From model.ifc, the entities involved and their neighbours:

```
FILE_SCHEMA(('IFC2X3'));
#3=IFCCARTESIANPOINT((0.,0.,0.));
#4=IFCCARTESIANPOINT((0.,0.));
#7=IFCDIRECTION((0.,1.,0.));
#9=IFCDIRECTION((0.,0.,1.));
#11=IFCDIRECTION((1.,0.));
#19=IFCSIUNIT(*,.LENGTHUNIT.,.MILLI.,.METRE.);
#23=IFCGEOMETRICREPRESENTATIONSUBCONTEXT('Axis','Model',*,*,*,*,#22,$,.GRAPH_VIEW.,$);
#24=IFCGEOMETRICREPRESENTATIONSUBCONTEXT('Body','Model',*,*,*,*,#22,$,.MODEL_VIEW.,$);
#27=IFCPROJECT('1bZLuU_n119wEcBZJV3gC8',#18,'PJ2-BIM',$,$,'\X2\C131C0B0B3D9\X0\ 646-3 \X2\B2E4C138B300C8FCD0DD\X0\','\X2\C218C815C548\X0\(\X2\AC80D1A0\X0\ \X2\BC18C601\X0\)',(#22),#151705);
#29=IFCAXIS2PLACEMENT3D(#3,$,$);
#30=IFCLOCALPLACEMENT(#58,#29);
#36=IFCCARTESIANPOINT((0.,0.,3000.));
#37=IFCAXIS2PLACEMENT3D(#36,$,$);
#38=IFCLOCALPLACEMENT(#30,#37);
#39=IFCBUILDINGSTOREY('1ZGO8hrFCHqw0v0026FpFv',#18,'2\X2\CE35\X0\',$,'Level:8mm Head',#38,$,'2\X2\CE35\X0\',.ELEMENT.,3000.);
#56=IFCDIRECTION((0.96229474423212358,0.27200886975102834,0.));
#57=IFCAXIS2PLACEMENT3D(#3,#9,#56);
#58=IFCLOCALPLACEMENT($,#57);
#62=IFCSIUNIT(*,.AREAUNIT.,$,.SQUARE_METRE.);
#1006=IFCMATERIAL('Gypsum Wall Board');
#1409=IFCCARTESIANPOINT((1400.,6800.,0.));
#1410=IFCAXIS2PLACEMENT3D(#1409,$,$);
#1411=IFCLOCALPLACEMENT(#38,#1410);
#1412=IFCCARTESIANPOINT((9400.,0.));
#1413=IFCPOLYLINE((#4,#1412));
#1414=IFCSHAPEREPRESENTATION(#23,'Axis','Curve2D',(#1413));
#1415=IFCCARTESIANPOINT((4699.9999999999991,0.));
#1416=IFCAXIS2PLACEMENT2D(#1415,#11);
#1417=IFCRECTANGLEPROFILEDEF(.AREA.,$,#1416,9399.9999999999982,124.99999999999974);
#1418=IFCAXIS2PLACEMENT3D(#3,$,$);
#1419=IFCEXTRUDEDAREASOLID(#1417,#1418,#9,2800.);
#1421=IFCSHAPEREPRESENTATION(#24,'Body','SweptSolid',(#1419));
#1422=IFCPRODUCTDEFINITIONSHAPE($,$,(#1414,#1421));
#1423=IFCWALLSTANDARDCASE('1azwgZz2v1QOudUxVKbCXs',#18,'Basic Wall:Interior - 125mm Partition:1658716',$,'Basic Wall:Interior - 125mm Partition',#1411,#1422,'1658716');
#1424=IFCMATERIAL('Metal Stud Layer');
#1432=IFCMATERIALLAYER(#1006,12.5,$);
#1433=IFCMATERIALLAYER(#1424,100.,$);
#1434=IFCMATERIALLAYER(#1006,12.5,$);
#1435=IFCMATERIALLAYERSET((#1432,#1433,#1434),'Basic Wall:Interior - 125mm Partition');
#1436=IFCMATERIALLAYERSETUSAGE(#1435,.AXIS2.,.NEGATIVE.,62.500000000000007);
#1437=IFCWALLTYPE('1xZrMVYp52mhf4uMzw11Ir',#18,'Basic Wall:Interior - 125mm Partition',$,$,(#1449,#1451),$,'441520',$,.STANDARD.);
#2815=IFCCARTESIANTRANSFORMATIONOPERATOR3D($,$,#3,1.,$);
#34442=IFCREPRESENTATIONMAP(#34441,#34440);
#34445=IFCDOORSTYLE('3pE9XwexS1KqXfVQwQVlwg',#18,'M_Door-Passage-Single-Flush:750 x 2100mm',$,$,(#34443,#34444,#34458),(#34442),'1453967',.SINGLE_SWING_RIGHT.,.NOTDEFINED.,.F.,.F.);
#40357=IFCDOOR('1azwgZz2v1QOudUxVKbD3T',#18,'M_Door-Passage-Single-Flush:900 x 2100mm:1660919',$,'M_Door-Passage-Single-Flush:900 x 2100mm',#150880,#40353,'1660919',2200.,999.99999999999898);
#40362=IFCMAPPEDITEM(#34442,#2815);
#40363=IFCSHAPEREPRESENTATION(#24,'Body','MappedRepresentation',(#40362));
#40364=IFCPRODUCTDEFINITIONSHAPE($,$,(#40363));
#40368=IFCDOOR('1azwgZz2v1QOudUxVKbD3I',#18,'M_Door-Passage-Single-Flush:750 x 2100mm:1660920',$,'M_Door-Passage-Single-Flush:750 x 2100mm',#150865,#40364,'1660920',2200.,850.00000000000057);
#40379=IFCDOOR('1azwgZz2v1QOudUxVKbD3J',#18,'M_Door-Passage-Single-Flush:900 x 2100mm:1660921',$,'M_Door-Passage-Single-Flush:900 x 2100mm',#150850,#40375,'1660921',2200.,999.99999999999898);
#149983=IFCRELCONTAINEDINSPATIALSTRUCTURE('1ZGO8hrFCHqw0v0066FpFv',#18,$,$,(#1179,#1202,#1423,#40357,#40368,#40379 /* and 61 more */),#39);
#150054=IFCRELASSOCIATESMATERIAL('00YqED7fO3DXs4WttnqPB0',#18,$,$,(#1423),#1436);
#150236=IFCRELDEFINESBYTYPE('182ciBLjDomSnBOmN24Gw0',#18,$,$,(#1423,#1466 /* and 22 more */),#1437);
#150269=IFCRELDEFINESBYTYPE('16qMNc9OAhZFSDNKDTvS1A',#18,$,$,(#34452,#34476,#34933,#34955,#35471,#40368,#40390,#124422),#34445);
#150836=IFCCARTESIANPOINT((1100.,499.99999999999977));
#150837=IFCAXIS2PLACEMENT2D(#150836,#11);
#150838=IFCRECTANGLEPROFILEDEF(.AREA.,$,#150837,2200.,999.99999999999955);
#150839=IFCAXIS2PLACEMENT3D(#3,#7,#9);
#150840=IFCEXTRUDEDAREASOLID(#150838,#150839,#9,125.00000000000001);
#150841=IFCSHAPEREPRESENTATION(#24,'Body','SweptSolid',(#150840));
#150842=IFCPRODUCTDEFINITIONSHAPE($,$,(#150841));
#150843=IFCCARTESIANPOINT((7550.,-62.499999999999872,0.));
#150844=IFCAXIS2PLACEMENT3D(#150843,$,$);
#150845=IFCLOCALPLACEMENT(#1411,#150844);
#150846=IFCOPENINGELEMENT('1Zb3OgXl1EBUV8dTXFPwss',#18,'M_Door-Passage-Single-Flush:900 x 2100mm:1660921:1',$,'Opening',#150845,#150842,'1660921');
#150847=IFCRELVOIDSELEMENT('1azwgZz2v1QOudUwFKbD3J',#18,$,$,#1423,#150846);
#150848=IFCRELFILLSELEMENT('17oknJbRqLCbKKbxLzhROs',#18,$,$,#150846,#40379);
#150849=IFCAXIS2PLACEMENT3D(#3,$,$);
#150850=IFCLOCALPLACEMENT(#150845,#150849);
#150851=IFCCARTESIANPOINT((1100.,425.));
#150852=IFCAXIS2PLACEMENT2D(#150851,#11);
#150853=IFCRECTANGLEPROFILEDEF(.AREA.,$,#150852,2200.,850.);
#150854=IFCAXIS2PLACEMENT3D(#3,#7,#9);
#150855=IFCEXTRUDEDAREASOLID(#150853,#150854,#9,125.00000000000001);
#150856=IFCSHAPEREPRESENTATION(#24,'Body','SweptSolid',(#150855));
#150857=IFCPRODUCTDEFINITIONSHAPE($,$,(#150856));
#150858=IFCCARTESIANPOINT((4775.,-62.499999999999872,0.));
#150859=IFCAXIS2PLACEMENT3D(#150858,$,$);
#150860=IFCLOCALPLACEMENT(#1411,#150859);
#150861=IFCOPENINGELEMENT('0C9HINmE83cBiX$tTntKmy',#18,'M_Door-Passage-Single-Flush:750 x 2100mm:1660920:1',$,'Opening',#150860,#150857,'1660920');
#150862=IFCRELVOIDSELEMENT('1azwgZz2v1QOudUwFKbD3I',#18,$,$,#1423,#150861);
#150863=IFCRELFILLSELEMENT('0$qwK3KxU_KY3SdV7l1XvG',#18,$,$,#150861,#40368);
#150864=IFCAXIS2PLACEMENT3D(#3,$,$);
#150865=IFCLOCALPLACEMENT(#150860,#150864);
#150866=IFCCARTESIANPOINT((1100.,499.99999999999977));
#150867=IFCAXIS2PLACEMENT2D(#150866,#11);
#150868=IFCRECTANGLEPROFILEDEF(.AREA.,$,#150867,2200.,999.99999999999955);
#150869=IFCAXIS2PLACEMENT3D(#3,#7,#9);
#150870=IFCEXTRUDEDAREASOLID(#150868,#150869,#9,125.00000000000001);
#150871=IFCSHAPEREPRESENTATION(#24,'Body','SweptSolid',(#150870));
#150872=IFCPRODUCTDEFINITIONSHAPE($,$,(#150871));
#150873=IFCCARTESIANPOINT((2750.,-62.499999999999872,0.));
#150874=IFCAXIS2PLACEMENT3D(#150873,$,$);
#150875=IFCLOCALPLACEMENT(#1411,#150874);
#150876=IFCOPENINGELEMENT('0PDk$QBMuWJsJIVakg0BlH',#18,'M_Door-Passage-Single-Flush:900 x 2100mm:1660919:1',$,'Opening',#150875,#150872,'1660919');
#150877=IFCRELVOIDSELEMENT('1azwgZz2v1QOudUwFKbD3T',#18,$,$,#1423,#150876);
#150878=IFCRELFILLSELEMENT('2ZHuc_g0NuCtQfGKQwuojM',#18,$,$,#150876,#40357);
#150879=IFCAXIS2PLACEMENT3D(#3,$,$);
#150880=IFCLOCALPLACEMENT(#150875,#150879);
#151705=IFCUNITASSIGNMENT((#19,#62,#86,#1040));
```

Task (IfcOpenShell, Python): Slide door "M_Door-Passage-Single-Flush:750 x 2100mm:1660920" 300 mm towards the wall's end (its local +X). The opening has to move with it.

```python
import ifcopenshell
import ifcopenshell.api.geometry
import ifcopenshell.util.placement
import ifcopenshell.util.unit

model = ifcopenshell.open("model.ifc")
unit_scale = ifcopenshell.util.unit.calculate_unit_scale(model)

door = model.by_guid("1azwgZz2v1QOudUxVKbD3I")
opening = door.FillsVoids[0].RelatingOpeningElement
wall = opening.VoidsElements[0].RelatingBuildingElement

wall_matrix = ifcopenshell.util.placement.get_local_placement(wall.ObjectPlacement)
shift = wall_matrix[:3, 0] * 0.3 / unit_scale
before = ifcopenshell.util.placement.get_local_placement(door.ObjectPlacement)[:3, 3].copy()

# The door is placed relative to its opening, so it follows when the opening moves.
matrix = ifcopenshell.util.placement.get_local_placement(opening.ObjectPlacement)
matrix[:3, 3] += shift
ifcopenshell.api.geometry.edit_object_placement(
    model, product=opening, matrix=matrix, is_si=False, should_transform_children=True
)

after = ifcopenshell.util.placement.get_local_placement(door.ObjectPlacement)[:3, 3]
print("door moved by", (after - before).round(3) + 0.0)

model.write("model_updated.ifc")
```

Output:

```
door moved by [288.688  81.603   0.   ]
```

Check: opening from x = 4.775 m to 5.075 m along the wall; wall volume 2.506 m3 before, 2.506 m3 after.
